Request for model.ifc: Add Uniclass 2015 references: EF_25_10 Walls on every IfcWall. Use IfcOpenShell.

First a look at what the model holds.

```python
import ifcopenshell

model = ifcopenshell.open("model.ifc")
print(model.schema)
print("classifications:", [c.Name for c in model.by_type("IfcClassification")])
for ifc_class in ("IfcDoor", "IfcRoof", "IfcStair", "IfcWall", "IfcWindow"):
    print(ifc_class, len(model.by_type(ifc_class)))
```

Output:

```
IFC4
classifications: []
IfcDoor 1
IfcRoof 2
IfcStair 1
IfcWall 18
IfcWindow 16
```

```python
import ifcopenshell
import ifcopenshell.api.classification

model = ifcopenshell.open("model.ifc")

system = ifcopenshell.api.classification.add_classification(model, classification="Uniclass 2015")

codes = {
    "IfcWall": ("EF_25_10", "Walls"),
}
for ifc_class, (code, name) in codes.items():
    products = model.by_type(ifc_class)
    ifcopenshell.api.classification.add_reference(
        model, products=products, classification=system, identification=code, name=name
    )
    print(code, len(products))

model.write("model-out.ifc")
```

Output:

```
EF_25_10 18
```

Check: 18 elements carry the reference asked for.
